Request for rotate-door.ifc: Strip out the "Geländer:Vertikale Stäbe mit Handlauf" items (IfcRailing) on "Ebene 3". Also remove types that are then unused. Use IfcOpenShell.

First a look at what the model holds.

```python
import ifcopenshell
import ifcopenshell.util.element

model = ifcopenshell.open("rotate-door.ifc")
print(model.schema)
storey = next(s for s in model.by_type("IfcBuildingStorey") if s.Name == "Ebene 3")
railings = [e for e in ifcopenshell.util.element.get_decomposition(storey) if e.is_a("IfcRailing")]
seen = {}
for e in railings:
    element_type = ifcopenshell.util.element.get_type(e)
    name = element_type.Name if element_type not in (None, e) else None
    seen[name] = seen.get(name, 0) + 1
for name, count in sorted(seen.items(), key=str):
    print(count, "x", name)
```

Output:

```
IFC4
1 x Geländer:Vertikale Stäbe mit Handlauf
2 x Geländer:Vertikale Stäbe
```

```python
import ifcopenshell
import ifcopenshell.api.root
import ifcopenshell.util.element

model = ifcopenshell.open("rotate-door.ifc")

storey = next(s for s in model.by_type("IfcBuildingStorey") if s.Name == "Ebene 3")
railings = [e for e in ifcopenshell.util.element.get_decomposition(storey) if e.is_a("IfcRailing")]
targets = [e for e in railings if (t := ifcopenshell.util.element.get_type(e)) not in (None, e) and t.Name == "Geländer:Vertikale Stäbe mit Handlauf"]
types = {ifcopenshell.util.element.get_type(e) for e in targets} - {None, *targets}

for e in targets:
    ifcopenshell.api.root.remove_product(model, product=e)
print(len(targets), "removed")

unused = [t for t in types if not ifcopenshell.util.element.get_types(t)]
for t in unused:
    ifcopenshell.api.root.remove_product(model, product=t)
print(len(unused), "unused types removed")

model.write("rotate-door-out.ifc")
```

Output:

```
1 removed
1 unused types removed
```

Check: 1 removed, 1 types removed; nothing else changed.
